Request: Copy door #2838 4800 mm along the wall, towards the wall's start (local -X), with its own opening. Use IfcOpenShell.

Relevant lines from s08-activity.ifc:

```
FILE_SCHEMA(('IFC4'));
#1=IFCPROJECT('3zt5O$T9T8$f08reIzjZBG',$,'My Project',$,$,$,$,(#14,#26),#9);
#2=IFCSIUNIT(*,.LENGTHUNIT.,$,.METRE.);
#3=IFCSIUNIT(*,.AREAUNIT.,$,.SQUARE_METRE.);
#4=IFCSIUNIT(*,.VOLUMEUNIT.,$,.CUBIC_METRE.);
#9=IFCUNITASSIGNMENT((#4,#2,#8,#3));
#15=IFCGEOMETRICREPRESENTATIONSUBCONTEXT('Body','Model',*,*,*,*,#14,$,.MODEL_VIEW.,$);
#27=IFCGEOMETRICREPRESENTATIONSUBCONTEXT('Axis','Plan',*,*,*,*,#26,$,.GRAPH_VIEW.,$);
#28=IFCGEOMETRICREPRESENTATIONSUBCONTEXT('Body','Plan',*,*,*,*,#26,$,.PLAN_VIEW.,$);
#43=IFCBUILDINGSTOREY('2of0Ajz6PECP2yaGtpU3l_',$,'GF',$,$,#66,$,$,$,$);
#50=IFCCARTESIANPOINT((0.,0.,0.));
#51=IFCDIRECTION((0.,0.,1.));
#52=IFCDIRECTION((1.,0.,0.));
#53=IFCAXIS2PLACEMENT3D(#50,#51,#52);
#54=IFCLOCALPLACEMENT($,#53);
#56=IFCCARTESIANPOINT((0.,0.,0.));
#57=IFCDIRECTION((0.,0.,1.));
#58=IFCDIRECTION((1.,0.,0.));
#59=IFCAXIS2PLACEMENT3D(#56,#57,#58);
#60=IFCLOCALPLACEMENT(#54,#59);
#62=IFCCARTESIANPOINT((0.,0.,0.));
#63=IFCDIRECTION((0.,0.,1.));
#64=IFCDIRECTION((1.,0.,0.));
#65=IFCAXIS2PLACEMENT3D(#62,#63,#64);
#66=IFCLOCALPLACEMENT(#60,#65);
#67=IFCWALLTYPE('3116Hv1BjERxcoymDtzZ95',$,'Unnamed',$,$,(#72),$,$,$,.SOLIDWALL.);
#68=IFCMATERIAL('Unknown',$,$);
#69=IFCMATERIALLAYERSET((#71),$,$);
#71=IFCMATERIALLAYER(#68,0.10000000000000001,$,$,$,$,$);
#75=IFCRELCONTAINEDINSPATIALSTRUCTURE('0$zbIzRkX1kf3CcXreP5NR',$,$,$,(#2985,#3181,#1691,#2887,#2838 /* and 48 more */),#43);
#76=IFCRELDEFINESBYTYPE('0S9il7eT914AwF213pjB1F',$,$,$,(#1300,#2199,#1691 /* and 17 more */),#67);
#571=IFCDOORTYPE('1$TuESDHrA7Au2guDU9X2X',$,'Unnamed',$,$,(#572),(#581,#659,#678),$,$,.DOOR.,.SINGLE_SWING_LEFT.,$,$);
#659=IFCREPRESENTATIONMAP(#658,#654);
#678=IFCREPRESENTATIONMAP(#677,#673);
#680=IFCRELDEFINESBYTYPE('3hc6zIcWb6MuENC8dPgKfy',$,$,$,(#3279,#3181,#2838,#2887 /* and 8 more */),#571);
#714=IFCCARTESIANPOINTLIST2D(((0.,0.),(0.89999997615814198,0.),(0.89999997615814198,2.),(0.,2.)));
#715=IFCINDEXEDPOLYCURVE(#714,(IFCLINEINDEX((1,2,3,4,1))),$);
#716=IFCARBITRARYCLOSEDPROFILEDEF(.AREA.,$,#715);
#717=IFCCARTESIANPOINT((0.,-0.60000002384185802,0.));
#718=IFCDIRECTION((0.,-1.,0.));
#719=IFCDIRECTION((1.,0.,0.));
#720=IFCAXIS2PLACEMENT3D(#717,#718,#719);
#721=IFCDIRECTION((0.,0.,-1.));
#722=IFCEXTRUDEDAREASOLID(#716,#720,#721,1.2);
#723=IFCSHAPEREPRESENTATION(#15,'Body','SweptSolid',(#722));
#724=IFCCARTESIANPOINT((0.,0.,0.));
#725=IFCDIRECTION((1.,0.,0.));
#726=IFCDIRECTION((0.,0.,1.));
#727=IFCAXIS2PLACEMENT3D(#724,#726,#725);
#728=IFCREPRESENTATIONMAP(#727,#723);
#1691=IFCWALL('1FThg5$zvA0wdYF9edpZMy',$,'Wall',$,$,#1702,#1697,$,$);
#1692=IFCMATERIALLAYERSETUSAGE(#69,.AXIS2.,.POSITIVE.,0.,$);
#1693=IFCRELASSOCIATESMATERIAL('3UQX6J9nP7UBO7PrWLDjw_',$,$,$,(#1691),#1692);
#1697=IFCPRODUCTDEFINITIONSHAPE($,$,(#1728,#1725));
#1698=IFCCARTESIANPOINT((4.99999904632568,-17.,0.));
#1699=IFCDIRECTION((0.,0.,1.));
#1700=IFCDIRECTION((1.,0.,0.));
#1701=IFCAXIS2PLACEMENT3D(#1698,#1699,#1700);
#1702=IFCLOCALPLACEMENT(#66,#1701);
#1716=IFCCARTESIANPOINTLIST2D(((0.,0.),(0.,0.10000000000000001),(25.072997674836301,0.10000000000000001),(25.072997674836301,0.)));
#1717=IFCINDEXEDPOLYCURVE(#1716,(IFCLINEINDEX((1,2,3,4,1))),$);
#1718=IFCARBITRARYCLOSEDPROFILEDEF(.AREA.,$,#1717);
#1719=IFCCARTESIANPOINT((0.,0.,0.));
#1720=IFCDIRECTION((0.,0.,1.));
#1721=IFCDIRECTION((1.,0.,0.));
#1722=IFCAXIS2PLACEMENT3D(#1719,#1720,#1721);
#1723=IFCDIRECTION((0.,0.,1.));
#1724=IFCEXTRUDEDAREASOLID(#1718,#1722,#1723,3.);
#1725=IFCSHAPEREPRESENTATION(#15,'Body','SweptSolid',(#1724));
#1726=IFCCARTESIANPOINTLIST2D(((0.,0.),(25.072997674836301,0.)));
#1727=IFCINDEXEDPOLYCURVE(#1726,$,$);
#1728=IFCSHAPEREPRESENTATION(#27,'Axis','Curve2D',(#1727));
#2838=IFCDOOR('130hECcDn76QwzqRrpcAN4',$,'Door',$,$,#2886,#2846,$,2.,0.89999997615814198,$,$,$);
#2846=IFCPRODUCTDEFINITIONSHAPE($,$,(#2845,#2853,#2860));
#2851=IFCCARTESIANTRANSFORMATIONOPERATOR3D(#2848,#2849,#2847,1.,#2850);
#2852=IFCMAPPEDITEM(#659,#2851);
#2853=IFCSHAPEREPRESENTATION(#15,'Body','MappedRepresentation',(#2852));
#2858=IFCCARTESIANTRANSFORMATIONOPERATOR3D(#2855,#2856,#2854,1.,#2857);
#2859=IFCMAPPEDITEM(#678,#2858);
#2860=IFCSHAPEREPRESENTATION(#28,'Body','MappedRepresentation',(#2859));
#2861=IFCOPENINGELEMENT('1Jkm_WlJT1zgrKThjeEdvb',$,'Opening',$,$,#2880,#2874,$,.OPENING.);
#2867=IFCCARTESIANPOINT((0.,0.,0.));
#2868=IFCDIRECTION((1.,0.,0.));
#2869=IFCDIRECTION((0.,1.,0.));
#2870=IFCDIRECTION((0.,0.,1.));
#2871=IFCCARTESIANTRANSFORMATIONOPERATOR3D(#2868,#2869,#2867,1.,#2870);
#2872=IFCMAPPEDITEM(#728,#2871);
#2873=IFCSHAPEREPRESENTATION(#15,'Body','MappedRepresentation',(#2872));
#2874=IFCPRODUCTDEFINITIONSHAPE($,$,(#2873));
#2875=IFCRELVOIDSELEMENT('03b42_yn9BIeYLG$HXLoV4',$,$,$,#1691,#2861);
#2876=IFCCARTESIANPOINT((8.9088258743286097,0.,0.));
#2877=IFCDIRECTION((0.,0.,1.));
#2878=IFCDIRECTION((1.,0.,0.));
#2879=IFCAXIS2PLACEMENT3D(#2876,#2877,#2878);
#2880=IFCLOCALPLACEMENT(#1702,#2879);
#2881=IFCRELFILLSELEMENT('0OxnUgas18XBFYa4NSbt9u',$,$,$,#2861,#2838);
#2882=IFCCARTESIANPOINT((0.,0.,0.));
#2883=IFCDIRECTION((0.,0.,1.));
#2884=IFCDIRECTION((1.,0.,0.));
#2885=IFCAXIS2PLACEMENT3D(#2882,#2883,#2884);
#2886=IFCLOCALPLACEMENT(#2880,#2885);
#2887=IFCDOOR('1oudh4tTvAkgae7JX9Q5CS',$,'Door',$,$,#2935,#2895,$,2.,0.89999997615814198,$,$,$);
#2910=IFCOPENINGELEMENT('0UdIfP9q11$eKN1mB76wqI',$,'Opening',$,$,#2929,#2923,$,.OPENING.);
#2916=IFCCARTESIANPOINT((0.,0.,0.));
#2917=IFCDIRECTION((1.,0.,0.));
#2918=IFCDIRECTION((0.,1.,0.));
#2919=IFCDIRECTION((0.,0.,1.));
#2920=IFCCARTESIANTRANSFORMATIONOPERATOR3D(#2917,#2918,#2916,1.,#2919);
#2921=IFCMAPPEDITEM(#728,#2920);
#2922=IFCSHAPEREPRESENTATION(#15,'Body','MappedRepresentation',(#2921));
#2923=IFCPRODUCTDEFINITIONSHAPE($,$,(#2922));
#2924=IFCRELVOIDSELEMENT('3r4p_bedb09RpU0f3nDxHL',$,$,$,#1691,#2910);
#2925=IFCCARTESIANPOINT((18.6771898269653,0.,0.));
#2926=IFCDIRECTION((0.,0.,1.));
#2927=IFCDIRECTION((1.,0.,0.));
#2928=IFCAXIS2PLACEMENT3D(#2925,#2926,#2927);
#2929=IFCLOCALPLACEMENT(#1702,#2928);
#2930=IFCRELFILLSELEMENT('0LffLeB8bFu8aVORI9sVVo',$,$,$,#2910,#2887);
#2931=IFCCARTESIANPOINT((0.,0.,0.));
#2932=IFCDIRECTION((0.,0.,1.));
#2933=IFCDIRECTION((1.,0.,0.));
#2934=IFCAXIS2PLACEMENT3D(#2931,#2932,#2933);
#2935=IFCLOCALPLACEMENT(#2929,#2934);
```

```python
import ifcopenshell
import ifcopenshell.api.feature
import ifcopenshell.api.geometry
import ifcopenshell.api.root
import ifcopenshell.geom
import ifcopenshell.util.element
import ifcopenshell.util.placement
import ifcopenshell.util.shape
import ifcopenshell.util.unit

model = ifcopenshell.open("s08-activity.ifc")
unit_scale = ifcopenshell.util.unit.calculate_unit_scale(model)
settings = ifcopenshell.geom.settings()


def volume(element):
    """Net volume in cubic metres, openings subtracted."""
    shape = ifcopenshell.geom.create_shape(settings, element)
    return ifcopenshell.util.shape.get_volume(shape.geometry)


door = model.by_id(2838)
opening = door.FillsVoids[0].RelatingOpeningElement
wall = opening.VoidsElements[0].RelatingBuildingElement
before = volume(wall)
shift = ifcopenshell.util.placement.get_local_placement(wall.ObjectPlacement)[:3, 0] * -4.8 / unit_scale

# copy_class copies the void relationship, type, container and properties, but no geometry.
new_opening = ifcopenshell.api.root.copy_class(model, product=opening)
new_opening.Representation = ifcopenshell.util.element.copy_deep(
    model, opening.Representation, exclude=["IfcGeometricRepresentationContext", "IfcRepresentationMap"]
)
new_door = ifcopenshell.api.root.copy_class(model, product=door)
new_door.Representation = ifcopenshell.util.element.copy_deep(
    model, door.Representation, exclude=["IfcGeometricRepresentationContext", "IfcRepresentationMap"]
)
ifcopenshell.api.feature.add_filling(model, opening=new_opening, element=new_door)

for old, new in ((opening, new_opening), (door, new_door)):
    matrix = ifcopenshell.util.placement.get_local_placement(old.ObjectPlacement)
    matrix[:3, 3] += shift
    ifcopenshell.api.geometry.edit_object_placement(model, product=new, matrix=matrix, is_si=False)

after = volume(wall)

print(f"wall volume {before:.3f} -> {after:.3f} m3")

model.write("s08-activity_edited.ifc")
```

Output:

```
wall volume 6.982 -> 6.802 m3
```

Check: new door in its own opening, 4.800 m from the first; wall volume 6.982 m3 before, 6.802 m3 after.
